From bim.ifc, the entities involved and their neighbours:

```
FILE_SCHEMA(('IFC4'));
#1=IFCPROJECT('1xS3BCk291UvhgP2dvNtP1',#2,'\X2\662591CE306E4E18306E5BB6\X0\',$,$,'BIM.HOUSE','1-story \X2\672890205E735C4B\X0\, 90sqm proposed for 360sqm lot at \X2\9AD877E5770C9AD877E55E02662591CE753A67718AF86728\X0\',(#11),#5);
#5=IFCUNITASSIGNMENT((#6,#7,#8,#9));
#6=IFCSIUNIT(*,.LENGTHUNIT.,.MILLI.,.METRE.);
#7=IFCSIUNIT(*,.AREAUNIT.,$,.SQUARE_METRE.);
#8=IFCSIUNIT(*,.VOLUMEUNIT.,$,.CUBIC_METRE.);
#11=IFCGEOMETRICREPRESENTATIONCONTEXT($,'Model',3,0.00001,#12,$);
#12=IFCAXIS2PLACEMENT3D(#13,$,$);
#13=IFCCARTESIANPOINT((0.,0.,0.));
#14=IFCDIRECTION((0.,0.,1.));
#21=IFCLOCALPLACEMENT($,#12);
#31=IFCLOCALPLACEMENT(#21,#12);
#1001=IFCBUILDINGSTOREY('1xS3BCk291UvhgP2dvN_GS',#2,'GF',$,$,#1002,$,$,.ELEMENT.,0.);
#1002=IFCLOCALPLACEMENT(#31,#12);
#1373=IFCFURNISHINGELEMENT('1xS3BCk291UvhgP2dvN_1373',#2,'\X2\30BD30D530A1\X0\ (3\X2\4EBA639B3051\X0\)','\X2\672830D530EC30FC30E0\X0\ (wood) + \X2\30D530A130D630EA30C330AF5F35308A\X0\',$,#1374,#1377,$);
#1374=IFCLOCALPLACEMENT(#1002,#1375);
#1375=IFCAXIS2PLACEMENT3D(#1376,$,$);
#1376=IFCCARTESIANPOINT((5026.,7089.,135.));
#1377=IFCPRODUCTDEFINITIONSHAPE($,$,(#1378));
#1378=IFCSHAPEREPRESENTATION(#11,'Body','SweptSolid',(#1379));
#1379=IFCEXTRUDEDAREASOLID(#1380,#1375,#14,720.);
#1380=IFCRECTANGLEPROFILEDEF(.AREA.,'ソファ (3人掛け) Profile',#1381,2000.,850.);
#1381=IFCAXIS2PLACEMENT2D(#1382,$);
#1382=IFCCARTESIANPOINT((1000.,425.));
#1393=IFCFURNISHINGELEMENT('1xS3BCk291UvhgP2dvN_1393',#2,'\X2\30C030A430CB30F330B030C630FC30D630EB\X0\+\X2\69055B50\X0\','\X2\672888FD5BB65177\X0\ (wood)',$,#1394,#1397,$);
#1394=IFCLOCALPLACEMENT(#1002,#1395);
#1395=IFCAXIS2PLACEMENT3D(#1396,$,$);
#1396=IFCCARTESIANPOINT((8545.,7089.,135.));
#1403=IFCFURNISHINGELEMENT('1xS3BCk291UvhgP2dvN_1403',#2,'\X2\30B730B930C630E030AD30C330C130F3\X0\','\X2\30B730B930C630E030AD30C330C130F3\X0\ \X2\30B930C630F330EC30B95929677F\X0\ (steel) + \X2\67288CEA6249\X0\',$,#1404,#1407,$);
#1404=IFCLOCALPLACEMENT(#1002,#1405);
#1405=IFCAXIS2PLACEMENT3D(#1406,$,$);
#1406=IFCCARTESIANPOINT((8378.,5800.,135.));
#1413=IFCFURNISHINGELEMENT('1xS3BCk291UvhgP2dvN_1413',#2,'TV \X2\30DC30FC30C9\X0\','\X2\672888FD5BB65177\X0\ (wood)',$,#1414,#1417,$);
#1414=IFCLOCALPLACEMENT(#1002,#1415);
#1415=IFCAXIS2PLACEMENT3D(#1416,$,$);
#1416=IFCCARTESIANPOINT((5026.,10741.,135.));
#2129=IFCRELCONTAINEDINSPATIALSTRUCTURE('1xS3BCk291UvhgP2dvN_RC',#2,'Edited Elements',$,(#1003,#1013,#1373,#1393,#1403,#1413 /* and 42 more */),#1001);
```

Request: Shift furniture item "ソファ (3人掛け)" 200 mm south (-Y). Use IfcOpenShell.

```python
import ifcopenshell
import ifcopenshell.api.geometry
import ifcopenshell.util.placement
import ifcopenshell.util.unit

model = ifcopenshell.open("bim.ifc")
unit_scale = ifcopenshell.util.unit.calculate_unit_scale(model)

item = model.by_guid("1xS3BCk291UvhgP2dvN_1373")
matrix = ifcopenshell.util.placement.get_local_placement(item.ObjectPlacement)
matrix[1, 3] -= 0.2 / unit_scale
ifcopenshell.api.geometry.edit_object_placement(model, product=item, matrix=matrix, is_si=False)

print(ifcopenshell.util.placement.get_local_placement(item.ObjectPlacement).round(3) + 0.0)

model.write("bim_v2.ifc")
```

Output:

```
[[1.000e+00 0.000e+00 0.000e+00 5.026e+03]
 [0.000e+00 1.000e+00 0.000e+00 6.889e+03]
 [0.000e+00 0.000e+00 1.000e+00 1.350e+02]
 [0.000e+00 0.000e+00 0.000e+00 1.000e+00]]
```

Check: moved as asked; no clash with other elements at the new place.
